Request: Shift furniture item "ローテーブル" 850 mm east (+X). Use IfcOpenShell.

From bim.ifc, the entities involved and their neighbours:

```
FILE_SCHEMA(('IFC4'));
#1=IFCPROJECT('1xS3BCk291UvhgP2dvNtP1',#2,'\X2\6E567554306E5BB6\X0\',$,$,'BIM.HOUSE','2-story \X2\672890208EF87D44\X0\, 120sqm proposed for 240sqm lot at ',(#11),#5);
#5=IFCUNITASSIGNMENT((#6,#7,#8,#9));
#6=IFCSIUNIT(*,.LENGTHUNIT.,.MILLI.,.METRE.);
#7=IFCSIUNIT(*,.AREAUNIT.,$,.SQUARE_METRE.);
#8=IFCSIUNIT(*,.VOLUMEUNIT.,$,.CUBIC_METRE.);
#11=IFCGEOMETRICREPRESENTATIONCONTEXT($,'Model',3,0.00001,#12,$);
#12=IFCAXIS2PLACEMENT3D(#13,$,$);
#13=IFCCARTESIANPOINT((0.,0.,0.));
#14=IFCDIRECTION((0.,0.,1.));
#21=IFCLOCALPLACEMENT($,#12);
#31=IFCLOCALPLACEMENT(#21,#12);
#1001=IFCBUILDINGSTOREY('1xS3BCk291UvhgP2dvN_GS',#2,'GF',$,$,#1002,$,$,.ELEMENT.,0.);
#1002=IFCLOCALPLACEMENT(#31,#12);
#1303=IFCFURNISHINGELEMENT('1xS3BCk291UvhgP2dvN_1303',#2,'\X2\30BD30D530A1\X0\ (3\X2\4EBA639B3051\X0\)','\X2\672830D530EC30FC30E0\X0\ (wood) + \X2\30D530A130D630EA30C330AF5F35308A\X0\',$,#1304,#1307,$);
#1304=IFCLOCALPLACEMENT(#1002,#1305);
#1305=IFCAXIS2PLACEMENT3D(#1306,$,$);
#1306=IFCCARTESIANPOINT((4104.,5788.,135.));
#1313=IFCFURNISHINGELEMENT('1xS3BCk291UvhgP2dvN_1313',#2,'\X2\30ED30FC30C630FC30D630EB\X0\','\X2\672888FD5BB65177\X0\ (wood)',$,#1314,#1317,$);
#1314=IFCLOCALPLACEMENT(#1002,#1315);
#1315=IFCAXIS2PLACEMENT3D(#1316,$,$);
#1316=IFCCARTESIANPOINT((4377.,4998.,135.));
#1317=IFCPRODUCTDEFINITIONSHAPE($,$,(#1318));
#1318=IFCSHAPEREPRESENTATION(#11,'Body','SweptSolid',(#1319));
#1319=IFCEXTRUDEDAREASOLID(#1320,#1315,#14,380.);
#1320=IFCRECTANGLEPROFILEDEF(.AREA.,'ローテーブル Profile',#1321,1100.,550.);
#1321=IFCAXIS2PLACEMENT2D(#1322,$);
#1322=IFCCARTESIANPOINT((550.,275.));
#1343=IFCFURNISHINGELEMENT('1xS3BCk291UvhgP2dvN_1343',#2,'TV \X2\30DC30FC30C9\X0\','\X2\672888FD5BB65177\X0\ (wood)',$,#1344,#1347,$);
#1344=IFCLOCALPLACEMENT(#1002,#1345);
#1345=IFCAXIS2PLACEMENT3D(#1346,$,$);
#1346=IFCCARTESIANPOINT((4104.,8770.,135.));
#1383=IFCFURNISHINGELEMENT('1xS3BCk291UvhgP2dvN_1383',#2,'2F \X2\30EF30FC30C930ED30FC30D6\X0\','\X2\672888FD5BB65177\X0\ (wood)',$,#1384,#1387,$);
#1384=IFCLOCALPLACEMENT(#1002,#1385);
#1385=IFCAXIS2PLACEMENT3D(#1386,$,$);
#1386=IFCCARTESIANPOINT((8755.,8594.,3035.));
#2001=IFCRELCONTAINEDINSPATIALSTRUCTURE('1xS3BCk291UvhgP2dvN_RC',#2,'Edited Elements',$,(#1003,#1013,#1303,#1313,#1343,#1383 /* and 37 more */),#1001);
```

```python
import ifcopenshell
import ifcopenshell.api.geometry
import ifcopenshell.util.placement
import ifcopenshell.util.unit

model = ifcopenshell.open("bim.ifc")
unit_scale = ifcopenshell.util.unit.calculate_unit_scale(model)

item = model.by_guid("1xS3BCk291UvhgP2dvN_1313")
matrix = ifcopenshell.util.placement.get_local_placement(item.ObjectPlacement)
matrix[0, 3] += 0.85 / unit_scale
ifcopenshell.api.geometry.edit_object_placement(model, product=item, matrix=matrix, is_si=False)

print(ifcopenshell.util.placement.get_local_placement(item.ObjectPlacement).round(3) + 0.0)

model.write("bim_v2.ifc")
```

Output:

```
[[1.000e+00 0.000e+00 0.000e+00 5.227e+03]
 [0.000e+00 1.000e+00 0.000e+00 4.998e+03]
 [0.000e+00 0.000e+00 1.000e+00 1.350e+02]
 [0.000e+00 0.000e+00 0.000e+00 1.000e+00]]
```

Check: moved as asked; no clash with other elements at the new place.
